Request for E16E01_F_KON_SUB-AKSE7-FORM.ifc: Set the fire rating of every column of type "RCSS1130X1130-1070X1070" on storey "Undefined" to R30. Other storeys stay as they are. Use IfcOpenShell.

First a look at what the model holds.

```python
import ifcopenshell
import ifcopenshell.util.element

model = ifcopenshell.open("E16E01_F_KON_SUB-AKSE7-FORM.ifc")
print(model.schema)
storey = next(s for s in model.by_type("IfcBuildingStorey") if s.Name == "Undefined")
columns = [e for e in ifcopenshell.util.element.get_decomposition(storey) if e.is_a("IfcColumn")]
seen = {}
for e in columns:
    element_type = ifcopenshell.util.element.get_type(e)
    key = (element_type.Name if element_type != e and element_type else None, ifcopenshell.util.element.get_pset(e, "Pset_ColumnCommon", "FireRating"))
    seen[key] = seen.get(key, 0) + 1
for (name, value), count in sorted(seen.items(), key=str):
    print(count, "x", name, "|", value)
```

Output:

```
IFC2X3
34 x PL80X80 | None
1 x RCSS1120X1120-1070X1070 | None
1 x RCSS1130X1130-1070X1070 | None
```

```python
import ifcopenshell
import ifcopenshell.api.pset
import ifcopenshell.util.element

model = ifcopenshell.open("E16E01_F_KON_SUB-AKSE7-FORM.ifc")

storey = next(s for s in model.by_type("IfcBuildingStorey") if s.Name == "Undefined")
columns = [e for e in ifcopenshell.util.element.get_decomposition(storey) if e.is_a("IfcColumn")]

count = 0
for e in columns:
    element_type = ifcopenshell.util.element.get_type(e)
    if element_type in (None, e) or element_type.Name != "RCSS1130X1130-1070X1070":
        continue
    # add_pset returns the element's existing set when there is one.
    pset = ifcopenshell.api.pset.add_pset(model, product=e, name="Pset_ColumnCommon")
    ifcopenshell.api.pset.edit_pset(model, pset=pset, properties={"FireRating": "R30"})
    count += 1

print(count, "columns updated")

model.write("E16E01_F_KON_SUB-AKSE7-FORM_rev.ifc")
```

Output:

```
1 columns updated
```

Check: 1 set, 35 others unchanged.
